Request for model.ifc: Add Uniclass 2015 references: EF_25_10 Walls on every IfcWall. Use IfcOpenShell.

First a look at what the model holds.

```python
import ifcopenshell

model = ifcopenshell.open("model.ifc")
print(model.schema)
print("classifications:", [c.Name for c in model.by_type("IfcClassification")])
for ifc_class in ("IfcDoor", "IfcRoof", "IfcStair", "IfcWall", "IfcWindow"):
    print(ifc_class, len(model.by_type(ifc_class)))
```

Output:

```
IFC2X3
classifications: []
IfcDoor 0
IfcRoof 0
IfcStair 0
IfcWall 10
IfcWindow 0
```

```python
import ifcopenshell
import ifcopenshell.api.classification

model = ifcopenshell.open("model.ifc")

# IFC2X3 requires Source and Edition and has no link from the project to the system.
system = model.create_entity("IfcClassification", Source="NBS", Edition="2015", Name="Uniclass 2015")

codes = {
    "IfcWall": ("EF_25_10", "Walls"),
}
for ifc_class, (code, name) in codes.items():
    products = model.by_type(ifc_class)
    ifcopenshell.api.classification.add_reference(
        model, products=products, classification=system, identification=code, name=name
    )
    print(code, len(products))

model.write("model_v2.ifc")
```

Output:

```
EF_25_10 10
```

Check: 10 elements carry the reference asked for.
